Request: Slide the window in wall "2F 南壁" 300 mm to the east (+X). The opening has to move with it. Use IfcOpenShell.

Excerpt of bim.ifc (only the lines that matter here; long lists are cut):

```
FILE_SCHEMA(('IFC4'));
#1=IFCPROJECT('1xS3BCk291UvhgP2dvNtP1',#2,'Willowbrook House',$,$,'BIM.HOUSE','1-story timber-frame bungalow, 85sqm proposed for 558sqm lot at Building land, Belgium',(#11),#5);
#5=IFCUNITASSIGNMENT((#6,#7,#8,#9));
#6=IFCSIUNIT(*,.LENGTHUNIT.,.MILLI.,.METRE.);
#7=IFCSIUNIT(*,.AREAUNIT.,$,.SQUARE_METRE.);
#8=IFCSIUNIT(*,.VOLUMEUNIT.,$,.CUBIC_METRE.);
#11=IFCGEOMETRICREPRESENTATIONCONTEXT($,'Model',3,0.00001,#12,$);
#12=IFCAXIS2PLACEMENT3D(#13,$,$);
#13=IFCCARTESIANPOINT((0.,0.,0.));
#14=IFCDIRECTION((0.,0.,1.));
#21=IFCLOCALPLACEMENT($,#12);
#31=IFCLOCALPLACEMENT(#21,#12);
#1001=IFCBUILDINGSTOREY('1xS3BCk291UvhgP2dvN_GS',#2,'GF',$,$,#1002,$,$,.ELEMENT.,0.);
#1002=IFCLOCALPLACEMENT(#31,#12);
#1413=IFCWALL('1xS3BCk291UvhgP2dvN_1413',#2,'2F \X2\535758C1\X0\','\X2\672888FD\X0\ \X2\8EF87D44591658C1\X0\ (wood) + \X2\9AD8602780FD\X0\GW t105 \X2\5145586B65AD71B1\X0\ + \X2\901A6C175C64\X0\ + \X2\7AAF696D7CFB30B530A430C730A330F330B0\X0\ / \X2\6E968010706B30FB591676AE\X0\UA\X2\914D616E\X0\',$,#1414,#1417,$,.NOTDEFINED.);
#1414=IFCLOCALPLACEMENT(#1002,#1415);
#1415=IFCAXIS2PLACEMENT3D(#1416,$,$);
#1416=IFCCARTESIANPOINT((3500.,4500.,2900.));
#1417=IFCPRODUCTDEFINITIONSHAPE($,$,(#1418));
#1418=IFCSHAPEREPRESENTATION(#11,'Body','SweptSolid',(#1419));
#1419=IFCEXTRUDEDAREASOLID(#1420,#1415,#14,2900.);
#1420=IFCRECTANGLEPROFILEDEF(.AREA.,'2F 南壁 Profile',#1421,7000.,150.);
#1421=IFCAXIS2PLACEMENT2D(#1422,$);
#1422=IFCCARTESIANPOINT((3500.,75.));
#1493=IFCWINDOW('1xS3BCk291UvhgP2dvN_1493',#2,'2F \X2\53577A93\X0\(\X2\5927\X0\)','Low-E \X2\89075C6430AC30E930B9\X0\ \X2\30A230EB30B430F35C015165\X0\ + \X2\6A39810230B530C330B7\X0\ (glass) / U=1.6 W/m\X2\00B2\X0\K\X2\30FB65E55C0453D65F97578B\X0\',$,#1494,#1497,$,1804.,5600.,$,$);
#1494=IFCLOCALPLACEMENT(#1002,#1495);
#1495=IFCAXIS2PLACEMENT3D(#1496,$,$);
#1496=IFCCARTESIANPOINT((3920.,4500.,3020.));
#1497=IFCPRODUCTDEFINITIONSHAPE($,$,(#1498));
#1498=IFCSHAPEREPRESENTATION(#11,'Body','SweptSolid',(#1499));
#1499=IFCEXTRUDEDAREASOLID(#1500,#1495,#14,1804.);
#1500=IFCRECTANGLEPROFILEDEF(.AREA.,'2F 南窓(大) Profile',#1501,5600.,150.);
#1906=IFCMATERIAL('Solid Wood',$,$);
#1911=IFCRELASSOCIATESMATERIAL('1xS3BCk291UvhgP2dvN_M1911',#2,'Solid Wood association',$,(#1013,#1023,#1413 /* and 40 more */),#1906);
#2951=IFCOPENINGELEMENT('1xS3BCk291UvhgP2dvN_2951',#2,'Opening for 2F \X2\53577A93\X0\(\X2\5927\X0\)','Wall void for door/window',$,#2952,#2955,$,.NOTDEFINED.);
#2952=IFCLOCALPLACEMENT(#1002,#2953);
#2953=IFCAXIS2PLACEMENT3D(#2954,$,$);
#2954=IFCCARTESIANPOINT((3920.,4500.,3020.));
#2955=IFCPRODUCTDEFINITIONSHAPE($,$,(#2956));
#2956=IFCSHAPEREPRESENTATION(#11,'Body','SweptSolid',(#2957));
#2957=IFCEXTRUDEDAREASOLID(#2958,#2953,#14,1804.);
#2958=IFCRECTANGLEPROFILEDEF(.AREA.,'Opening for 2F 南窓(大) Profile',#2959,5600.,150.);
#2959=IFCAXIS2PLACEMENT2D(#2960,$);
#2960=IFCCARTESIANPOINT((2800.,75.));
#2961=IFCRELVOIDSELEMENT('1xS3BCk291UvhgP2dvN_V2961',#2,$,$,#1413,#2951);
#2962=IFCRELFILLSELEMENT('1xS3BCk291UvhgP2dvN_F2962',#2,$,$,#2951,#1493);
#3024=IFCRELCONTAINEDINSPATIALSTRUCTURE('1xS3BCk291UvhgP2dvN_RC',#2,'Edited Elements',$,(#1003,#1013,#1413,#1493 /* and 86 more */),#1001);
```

```python
import ifcopenshell
import ifcopenshell.api.geometry
import ifcopenshell.util.placement
import ifcopenshell.util.unit

model = ifcopenshell.open("bim.ifc")
unit_scale = ifcopenshell.util.unit.calculate_unit_scale(model)

window = model.by_id(1493)
opening = window.FillsVoids[0].RelatingOpeningElement
wall = opening.VoidsElements[0].RelatingBuildingElement

wall_matrix = ifcopenshell.util.placement.get_local_placement(wall.ObjectPlacement)
shift = wall_matrix[:3, 0] * 0.3 / unit_scale
before = ifcopenshell.util.placement.get_local_placement(window.ObjectPlacement)[:3, 3].copy()

# The window is not placed relative to its opening, so move both.
for product in (opening, window):
    matrix = ifcopenshell.util.placement.get_local_placement(product.ObjectPlacement)
    matrix[:3, 3] += shift
    ifcopenshell.api.geometry.edit_object_placement(model, product=product, matrix=matrix, is_si=False)

after = ifcopenshell.util.placement.get_local_placement(window.ObjectPlacement)[:3, 3]
print("window moved by", (after - before).round(3) + 0.0)

model.write("bim_v2.ifc")
```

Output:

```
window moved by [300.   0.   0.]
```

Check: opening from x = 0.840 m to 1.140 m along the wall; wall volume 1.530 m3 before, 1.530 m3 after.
